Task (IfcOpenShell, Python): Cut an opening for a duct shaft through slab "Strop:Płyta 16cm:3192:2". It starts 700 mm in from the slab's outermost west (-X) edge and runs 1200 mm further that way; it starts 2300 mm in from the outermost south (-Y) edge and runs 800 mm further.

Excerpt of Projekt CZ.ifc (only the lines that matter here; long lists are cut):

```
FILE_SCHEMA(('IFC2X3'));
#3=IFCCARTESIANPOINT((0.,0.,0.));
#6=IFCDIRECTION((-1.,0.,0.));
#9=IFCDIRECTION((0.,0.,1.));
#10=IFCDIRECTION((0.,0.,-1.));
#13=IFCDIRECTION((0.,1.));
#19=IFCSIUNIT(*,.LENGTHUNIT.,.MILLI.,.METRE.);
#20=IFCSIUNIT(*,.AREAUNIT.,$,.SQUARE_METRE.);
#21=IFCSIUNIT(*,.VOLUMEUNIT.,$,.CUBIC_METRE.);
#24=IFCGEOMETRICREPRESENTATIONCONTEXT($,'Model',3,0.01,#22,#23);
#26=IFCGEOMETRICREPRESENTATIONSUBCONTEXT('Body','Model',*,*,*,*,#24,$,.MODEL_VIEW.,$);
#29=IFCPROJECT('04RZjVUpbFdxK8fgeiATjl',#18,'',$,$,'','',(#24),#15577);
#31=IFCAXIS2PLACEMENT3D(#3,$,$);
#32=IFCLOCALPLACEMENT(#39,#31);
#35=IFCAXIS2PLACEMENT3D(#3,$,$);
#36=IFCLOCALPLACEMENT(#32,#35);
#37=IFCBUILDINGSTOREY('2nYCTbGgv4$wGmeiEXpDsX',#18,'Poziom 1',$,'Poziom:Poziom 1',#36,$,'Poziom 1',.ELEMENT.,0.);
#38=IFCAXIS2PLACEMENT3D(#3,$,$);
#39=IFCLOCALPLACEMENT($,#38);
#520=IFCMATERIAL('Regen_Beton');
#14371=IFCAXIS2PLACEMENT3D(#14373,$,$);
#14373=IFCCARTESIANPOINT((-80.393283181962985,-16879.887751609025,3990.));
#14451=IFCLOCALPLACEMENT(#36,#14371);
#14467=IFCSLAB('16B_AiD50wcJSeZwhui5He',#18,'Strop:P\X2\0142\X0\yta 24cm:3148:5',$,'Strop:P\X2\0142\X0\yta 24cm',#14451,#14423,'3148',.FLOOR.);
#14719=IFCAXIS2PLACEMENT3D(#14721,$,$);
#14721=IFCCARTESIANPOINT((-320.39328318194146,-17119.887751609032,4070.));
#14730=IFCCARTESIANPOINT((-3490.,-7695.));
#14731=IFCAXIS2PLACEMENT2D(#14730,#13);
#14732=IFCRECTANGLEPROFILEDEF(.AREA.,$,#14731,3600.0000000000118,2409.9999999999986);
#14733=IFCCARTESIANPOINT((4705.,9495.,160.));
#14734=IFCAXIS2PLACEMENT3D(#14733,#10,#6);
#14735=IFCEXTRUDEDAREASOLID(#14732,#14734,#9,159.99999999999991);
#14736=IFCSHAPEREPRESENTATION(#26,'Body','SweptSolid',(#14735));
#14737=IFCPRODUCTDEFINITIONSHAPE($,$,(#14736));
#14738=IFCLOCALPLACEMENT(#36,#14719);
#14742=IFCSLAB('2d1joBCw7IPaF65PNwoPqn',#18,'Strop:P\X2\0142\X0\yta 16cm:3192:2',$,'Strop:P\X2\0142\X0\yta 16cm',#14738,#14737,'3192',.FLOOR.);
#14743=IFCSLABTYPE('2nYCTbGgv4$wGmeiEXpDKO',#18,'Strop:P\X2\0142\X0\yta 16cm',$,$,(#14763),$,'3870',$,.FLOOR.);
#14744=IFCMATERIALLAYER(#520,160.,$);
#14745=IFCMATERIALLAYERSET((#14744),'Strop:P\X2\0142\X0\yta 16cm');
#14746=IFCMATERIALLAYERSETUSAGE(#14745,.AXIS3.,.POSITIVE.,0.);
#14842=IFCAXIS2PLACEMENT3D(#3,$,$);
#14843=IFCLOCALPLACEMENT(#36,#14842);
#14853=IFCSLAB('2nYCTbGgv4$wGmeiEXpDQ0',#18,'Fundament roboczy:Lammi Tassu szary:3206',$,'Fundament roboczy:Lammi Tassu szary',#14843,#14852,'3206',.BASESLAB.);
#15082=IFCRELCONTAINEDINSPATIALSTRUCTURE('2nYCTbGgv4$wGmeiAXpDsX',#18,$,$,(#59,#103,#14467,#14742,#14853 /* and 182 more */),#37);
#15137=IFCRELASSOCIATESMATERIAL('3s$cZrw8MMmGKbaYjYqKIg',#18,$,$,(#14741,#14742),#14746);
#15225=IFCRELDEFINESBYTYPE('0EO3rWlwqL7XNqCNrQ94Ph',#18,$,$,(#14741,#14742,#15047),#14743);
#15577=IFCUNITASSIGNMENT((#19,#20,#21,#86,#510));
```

```python
import numpy as np
import ifcopenshell
import ifcopenshell.api.feature
import ifcopenshell.api.geometry
import ifcopenshell.api.root
import ifcopenshell.geom
import ifcopenshell.util.placement
import ifcopenshell.util.representation
import ifcopenshell.util.shape
import ifcopenshell.util.unit

model = ifcopenshell.open("Projekt CZ.ifc")
unit_scale = ifcopenshell.util.unit.calculate_unit_scale(model)
settings = ifcopenshell.geom.settings()


def volume(element):
    """Net volume in cubic metres, openings subtracted."""
    shape = ifcopenshell.geom.create_shape(settings, element)
    return ifcopenshell.util.shape.get_volume(shape.geometry)


slab = model.by_id(14742)
before = volume(slab)

# Extent in the slab's own axes, in metres. The edges named are its -X and -Y sides.
slab_shape = ifcopenshell.geom.create_shape(settings, slab)
vertices = ifcopenshell.util.shape.get_vertices(slab_shape.geometry)
x_min, y_min, bottom = vertices.min(axis=0)
top = vertices[:, 2].max()

opening = ifcopenshell.api.root.create_entity(model, ifc_class="IfcOpeningElement", name="Duct shaft opening")
context = ifcopenshell.util.representation.get_context(model, "Model", "Body", "MODEL_VIEW")
width, depth = 1.2, 0.8
outline = [(0.0, 0.0), (width, 0.0), (width, depth), (0.0, depth), (0.0, 0.0)]
# Overshoot both faces by 50 mm so the cut is clean.
shape = ifcopenshell.api.geometry.add_slab_representation(
    model, context=context, depth=top - bottom + 0.1, polyline=outline
)
ifcopenshell.api.geometry.assign_representation(model, product=opening, representation=shape)

matrix = ifcopenshell.util.placement.get_local_placement(slab.ObjectPlacement)
matrix[:, 3] = matrix @ np.append(np.array([x_min + 0.7, y_min + 2.3, bottom - 0.05]) / unit_scale, 1.0)
ifcopenshell.api.geometry.edit_object_placement(model, product=opening, matrix=matrix, is_si=False)
ifcopenshell.api.feature.add_feature(model, feature=opening, element=slab)

after = volume(slab)

print(f"slab volume {before:.3f} -> {after:.3f} m3")

model.write("Projekt CZ-out.ifc")
```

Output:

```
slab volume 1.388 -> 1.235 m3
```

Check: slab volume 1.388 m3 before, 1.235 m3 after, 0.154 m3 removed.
